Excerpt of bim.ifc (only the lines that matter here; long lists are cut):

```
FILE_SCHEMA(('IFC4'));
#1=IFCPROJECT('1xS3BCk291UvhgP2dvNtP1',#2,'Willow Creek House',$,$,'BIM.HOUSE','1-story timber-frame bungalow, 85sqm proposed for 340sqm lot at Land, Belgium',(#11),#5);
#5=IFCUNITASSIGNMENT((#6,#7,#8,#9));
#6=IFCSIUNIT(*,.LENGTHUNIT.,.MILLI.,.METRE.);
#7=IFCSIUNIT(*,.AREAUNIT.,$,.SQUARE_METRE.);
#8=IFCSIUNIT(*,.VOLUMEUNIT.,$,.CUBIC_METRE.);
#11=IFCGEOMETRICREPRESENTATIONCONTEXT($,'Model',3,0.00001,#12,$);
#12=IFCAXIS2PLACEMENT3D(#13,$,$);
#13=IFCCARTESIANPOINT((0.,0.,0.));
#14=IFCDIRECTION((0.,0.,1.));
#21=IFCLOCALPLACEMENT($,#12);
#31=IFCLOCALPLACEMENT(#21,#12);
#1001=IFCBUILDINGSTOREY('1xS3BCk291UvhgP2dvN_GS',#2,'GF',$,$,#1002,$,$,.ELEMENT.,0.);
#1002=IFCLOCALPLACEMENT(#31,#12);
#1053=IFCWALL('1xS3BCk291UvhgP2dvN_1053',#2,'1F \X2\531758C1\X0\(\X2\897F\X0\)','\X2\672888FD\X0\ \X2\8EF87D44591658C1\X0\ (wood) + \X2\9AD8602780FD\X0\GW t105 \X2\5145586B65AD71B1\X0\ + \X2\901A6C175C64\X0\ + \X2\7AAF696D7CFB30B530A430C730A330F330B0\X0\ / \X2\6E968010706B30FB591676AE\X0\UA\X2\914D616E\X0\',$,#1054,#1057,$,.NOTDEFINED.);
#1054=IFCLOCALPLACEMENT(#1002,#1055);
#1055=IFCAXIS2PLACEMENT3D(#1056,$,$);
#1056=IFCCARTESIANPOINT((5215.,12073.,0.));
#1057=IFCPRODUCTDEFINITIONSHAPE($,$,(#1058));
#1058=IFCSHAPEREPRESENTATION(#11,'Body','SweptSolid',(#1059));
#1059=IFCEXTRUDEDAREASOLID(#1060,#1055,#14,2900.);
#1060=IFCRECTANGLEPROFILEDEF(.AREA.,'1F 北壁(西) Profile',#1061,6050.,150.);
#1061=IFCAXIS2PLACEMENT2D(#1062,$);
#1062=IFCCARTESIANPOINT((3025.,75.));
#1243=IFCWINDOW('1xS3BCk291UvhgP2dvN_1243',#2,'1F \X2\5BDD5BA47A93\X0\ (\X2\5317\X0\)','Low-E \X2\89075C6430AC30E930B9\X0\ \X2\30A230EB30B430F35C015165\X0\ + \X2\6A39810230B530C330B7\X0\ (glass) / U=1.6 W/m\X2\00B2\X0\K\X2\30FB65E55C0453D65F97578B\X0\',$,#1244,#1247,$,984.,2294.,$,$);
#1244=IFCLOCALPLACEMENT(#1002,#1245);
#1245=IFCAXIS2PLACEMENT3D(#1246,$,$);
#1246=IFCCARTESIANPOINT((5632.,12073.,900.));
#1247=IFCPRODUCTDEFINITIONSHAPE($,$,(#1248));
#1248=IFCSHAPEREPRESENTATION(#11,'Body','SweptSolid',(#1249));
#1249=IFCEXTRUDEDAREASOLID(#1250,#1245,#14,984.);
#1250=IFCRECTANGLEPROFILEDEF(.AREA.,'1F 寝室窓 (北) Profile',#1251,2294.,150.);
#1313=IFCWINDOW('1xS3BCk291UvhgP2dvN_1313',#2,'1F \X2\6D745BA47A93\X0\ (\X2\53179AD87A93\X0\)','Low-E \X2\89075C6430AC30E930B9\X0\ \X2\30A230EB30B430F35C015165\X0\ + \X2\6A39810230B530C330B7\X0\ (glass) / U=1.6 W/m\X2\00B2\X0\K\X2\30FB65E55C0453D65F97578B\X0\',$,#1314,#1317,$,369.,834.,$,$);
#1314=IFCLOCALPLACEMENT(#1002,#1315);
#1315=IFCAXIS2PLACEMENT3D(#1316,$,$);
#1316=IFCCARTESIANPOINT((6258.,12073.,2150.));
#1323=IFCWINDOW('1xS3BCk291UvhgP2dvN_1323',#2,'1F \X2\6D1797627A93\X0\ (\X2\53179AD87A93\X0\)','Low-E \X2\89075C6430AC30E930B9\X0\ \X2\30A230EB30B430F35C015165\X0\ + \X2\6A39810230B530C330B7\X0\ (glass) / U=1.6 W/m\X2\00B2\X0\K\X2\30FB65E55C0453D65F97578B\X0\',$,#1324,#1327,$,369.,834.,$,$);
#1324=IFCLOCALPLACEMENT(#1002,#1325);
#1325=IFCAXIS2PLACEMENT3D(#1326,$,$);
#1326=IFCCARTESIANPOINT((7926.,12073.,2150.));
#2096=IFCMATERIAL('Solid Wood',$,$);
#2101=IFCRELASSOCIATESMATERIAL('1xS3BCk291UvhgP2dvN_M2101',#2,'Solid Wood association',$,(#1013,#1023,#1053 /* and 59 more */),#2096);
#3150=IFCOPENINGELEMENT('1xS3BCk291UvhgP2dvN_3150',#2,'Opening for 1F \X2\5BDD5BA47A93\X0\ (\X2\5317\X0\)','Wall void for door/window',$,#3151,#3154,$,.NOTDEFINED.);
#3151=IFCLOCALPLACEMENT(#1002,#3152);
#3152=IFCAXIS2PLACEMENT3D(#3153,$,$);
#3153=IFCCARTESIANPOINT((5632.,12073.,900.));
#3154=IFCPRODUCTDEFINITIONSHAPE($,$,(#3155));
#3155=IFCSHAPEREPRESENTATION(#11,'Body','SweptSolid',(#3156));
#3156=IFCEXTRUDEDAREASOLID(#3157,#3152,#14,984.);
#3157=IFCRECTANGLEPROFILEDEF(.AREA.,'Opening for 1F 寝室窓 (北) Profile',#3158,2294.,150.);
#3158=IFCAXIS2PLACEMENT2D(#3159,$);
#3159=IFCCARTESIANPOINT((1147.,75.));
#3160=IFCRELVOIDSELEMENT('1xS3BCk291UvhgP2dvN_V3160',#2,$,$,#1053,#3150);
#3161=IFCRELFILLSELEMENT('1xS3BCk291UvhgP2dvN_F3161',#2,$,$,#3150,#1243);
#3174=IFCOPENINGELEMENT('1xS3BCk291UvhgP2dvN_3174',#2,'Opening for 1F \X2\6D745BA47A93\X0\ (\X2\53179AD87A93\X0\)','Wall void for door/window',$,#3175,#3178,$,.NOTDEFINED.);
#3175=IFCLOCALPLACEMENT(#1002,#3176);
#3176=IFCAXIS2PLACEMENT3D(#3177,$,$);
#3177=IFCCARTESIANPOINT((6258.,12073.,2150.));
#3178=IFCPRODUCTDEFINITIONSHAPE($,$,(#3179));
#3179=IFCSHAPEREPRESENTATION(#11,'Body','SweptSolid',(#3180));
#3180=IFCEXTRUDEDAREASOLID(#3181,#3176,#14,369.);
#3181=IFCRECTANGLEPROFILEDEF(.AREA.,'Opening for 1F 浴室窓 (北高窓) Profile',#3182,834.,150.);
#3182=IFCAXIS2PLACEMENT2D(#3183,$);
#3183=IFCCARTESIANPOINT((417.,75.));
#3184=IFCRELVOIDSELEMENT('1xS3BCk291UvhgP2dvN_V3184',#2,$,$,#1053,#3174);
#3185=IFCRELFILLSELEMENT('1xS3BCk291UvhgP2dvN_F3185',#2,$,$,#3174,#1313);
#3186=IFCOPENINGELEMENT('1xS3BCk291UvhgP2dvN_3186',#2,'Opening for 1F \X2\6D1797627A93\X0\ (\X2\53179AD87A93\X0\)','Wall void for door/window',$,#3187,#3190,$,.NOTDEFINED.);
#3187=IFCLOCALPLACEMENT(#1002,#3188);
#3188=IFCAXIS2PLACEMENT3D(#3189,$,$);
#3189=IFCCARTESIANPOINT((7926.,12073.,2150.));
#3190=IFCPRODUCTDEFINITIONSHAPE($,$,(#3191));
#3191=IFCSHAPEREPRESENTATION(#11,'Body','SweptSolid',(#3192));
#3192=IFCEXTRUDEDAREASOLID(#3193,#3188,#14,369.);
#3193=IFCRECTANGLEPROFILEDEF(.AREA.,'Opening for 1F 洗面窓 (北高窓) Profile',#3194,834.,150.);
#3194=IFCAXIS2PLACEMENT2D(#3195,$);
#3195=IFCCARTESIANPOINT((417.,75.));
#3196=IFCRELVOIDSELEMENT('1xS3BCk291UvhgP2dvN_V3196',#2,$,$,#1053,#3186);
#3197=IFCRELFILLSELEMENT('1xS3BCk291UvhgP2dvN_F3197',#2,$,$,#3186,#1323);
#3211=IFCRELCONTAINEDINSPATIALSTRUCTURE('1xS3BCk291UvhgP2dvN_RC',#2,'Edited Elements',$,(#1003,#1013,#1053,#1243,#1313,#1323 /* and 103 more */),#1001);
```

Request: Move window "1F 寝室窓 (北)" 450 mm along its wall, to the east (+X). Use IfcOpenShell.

```python
import ifcopenshell
import ifcopenshell.api.geometry
import ifcopenshell.util.placement

model = ifcopenshell.open("bim.ifc")

window = model.by_guid("1xS3BCk291UvhgP2dvN_1243")
opening = window.FillsVoids[0].RelatingOpeningElement
wall = opening.VoidsElements[0].RelatingBuildingElement

wall_matrix = ifcopenshell.util.placement.get_local_placement(wall.ObjectPlacement)
shift = wall_matrix[:3, 0] * 450.0
before = ifcopenshell.util.placement.get_local_placement(window.ObjectPlacement)[:3, 3].copy()

# The window is not placed relative to its opening, so move both.
for product in (opening, window):
    matrix = ifcopenshell.util.placement.get_local_placement(product.ObjectPlacement)
    matrix[:3, 3] += shift
    ifcopenshell.api.geometry.edit_object_placement(model, product=product, matrix=matrix, is_si=False)

after = ifcopenshell.util.placement.get_local_placement(window.ObjectPlacement)[:3, 3]
print("window moved by", (after - before).round(3) + 0.0)

model.write("bim_edited.ifc")
```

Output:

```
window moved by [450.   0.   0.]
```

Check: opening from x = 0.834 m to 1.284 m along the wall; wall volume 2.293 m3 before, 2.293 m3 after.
